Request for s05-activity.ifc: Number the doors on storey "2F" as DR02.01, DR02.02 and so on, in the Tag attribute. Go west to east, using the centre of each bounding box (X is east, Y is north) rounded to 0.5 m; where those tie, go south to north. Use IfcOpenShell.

First a look at what the model holds.

```python
import ifcopenshell
import ifcopenshell.util.element
import ifcopenshell.util.placement

model = ifcopenshell.open("s05-activity.ifc")
print(model.schema)
storey = next(s for s in model.by_type("IfcBuildingStorey") if s.Name == "2F")
doors = [e for e in ifcopenshell.util.element.get_decomposition(storey) if e.is_a("IfcDoor")]
for e in sorted(doors, key=lambda e: e.id()):
    origin = ifcopenshell.util.placement.get_local_placement(e.ObjectPlacement)[:3, 3]
    print(e.id(), e.Tag, e.Name, origin.round(2) + 0.0, sep=" | ")
```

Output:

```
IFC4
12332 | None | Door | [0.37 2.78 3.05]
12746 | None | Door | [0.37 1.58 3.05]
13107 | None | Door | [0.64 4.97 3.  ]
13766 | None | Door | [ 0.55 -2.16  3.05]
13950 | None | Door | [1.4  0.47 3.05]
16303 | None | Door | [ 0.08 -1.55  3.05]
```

```python
import ifcopenshell
import ifcopenshell.geom
import ifcopenshell.util.element
import ifcopenshell.util.shape

model = ifcopenshell.open("s05-activity.ifc")
settings = ifcopenshell.geom.settings()
settings.set("use-world-coords", True)


def centre(element):
    shape = ifcopenshell.geom.create_shape(settings, element)
    return ifcopenshell.util.shape.get_bbox_centroid(shape.geometry)


storey = next(s for s in model.by_type("IfcBuildingStorey") if s.Name == "2F")
doors = [e for e in ifcopenshell.util.element.get_decomposition(storey) if e.is_a("IfcDoor")]

# Insertion points can sit at a corner or the storey origin, so sort by the geometry (in metres).
centres = {e: centre(e) for e in doors}
doors.sort(key=lambda e: (round(centres[e][0] / 0.5), centres[e][1]))

for i, e in enumerate(doors, start=1):
    number = f"DR02.{i:02d}"
    e.Tag = number
    print(e.id(), number)

model.write("s05-activity_v2.ifc")
```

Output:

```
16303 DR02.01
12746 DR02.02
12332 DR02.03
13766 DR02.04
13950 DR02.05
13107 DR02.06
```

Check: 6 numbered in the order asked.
